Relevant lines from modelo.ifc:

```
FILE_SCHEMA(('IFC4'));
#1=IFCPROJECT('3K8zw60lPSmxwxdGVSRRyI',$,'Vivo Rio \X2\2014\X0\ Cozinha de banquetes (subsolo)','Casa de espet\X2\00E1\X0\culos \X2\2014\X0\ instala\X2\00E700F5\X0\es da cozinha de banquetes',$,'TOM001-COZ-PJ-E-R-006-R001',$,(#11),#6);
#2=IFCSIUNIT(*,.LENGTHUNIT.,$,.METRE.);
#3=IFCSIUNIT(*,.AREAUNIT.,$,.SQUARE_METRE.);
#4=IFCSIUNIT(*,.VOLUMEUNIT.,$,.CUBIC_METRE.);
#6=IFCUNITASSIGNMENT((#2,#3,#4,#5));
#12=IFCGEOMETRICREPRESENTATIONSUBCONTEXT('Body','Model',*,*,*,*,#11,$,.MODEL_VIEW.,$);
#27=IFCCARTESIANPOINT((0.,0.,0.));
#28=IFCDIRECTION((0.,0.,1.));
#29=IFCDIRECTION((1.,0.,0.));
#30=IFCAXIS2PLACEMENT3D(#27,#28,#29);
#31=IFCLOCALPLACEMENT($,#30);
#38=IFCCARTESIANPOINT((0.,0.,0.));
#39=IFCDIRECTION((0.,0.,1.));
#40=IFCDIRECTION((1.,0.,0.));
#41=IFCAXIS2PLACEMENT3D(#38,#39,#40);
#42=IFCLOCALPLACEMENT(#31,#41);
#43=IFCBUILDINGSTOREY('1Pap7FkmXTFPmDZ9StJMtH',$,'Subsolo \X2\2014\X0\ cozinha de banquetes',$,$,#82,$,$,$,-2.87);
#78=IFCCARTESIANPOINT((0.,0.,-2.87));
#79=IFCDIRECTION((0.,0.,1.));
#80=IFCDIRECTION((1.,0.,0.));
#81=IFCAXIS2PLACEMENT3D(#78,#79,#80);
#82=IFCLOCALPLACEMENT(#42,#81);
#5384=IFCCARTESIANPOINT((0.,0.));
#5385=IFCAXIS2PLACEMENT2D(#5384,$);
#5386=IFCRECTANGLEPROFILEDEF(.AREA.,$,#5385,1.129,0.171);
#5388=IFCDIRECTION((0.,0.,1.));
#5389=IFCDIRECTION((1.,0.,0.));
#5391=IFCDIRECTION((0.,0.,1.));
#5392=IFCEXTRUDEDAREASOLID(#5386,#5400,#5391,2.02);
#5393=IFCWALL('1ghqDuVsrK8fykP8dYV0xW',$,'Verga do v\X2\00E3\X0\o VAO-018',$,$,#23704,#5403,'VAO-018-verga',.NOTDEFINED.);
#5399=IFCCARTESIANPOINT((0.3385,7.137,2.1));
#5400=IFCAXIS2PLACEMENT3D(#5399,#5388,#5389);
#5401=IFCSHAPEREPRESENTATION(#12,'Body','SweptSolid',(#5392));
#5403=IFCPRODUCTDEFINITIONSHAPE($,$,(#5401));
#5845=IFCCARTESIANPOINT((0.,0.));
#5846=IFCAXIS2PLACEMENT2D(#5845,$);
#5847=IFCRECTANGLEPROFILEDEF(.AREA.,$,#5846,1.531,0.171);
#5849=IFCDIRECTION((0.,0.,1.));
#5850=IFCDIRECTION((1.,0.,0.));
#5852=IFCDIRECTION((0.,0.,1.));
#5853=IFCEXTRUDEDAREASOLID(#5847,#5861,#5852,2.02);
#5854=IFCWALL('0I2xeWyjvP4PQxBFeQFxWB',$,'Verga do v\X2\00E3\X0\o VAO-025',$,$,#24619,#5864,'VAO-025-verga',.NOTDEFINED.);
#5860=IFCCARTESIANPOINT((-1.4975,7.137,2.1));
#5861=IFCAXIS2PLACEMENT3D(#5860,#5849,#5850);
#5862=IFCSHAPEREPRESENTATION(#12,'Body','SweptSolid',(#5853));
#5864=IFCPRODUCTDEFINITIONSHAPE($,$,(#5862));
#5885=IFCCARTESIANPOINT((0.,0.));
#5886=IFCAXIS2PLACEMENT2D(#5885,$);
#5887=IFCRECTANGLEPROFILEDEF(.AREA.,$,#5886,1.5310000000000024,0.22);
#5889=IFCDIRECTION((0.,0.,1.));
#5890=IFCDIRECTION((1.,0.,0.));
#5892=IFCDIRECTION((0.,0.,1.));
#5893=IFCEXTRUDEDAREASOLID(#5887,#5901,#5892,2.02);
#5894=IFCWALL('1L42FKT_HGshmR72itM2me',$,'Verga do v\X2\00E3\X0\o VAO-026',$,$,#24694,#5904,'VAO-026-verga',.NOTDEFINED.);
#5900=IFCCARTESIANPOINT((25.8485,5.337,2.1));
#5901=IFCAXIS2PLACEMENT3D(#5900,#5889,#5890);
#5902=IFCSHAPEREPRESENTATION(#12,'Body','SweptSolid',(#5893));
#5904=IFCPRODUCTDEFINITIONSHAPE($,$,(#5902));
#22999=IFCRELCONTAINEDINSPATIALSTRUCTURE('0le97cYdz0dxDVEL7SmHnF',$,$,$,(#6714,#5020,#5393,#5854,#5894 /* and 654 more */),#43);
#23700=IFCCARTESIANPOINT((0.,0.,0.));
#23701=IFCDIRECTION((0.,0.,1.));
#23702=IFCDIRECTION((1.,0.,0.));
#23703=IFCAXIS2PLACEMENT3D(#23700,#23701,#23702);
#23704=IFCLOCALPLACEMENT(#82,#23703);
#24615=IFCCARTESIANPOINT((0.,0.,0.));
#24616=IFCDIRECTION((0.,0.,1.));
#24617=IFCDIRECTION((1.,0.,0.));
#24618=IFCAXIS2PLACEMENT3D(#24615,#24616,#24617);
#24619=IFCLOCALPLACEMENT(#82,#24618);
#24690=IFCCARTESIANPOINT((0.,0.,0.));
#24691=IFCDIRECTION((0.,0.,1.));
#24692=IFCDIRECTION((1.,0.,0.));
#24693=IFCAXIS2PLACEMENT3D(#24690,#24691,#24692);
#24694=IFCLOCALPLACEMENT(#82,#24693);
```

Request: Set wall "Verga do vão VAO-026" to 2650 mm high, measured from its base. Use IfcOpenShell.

```python
import ifcopenshell
import ifcopenshell.geom
import ifcopenshell.util.representation
import ifcopenshell.util.shape
import ifcopenshell.util.unit

model = ifcopenshell.open("modelo.ifc")
unit_scale = ifcopenshell.util.unit.calculate_unit_scale(model)
settings = ifcopenshell.geom.settings()


def volume(element):
    """Net volume in cubic metres, openings subtracted."""
    shape = ifcopenshell.geom.create_shape(settings, element)
    return ifcopenshell.util.shape.get_volume(shape.geometry)


wall = model.by_id(5894)
before = volume(wall)

body = ifcopenshell.util.representation.get_representation(wall, "Model", "Body")
solid = body.Items[0]
old_height = solid.Depth
solid.Depth = 2.65 / unit_scale
after = volume(wall)

print(f"height {old_height:g} -> {solid.Depth:g}, volume {before:.3f} -> {after:.3f} m3")

model.write("modelo-out.ifc")
```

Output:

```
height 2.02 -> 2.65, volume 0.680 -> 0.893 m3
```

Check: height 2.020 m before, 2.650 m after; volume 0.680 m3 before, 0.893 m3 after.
